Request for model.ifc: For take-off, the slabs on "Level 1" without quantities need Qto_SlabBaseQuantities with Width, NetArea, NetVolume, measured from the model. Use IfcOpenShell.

First a look at what the model holds.

```python
import ifcopenshell
import ifcopenshell.util.element
import ifcopenshell.util.unit

model = ifcopenshell.open("model.ifc")
print(model.schema)
for unit_type in ("LENGTHUNIT", "AREAUNIT", "VOLUMEUNIT"):
    print(unit_type, ifcopenshell.util.unit.calculate_unit_scale(model, unit_type))
storey = next(s for s in model.by_type("IfcBuildingStorey") if s.Name == "Level 1")
slabs = [e for e in ifcopenshell.util.element.get_decomposition(storey) if e.is_a("IfcSlab")]
for e in sorted(slabs, key=lambda e: e.id()):
    print(e.id(), e.is_a(), e.Name, list(ifcopenshell.util.element.get_psets(e, qtos_only=True)), sep=" | ")
```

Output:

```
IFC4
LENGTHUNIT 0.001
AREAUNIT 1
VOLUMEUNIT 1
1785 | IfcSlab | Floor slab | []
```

```python
import ifcopenshell
import ifcopenshell.api.pset
import ifcopenshell.geom
import ifcopenshell.util.element
import ifcopenshell.util.shape
import ifcopenshell.util.unit

model = ifcopenshell.open("model.ifc")
unit_scale = ifcopenshell.util.unit.calculate_unit_scale(model)
area_scale = ifcopenshell.util.unit.calculate_unit_scale(model, "AREAUNIT")
volume_scale = ifcopenshell.util.unit.calculate_unit_scale(model, "VOLUMEUNIT")
settings = ifcopenshell.geom.settings()

storey = next(s for s in model.by_type("IfcBuildingStorey") if s.Name == "Level 1")
slabs = [e for e in ifcopenshell.util.element.get_decomposition(storey) if e.is_a("IfcSlab")]

for e in sorted(slabs, key=lambda e: e.id()):
    if ifcopenshell.util.element.get_psets(e, qtos_only=True, should_inherit=False):
        continue
    # Geometry comes back in metres, in the element's own axes.
    shape = ifcopenshell.geom.create_shape(settings, e)
    values = {
        "Width": ifcopenshell.util.shape.get_z(shape.geometry) / unit_scale,
        "NetArea": ifcopenshell.util.shape.get_footprint_area(shape.geometry) / area_scale,
        "NetVolume": ifcopenshell.util.shape.get_volume(shape.geometry) / volume_scale,
    }
    qto = ifcopenshell.api.pset.add_qto(model, product=e, name="Qto_SlabBaseQuantities")
    ifcopenshell.api.pset.edit_qto(model, qto=qto, properties=values)
    print(e.id(), {k: round(v, 3) for k, v in values.items()})

model.write("model_edited.ifc")
```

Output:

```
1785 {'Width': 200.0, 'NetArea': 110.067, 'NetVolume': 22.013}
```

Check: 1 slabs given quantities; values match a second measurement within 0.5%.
